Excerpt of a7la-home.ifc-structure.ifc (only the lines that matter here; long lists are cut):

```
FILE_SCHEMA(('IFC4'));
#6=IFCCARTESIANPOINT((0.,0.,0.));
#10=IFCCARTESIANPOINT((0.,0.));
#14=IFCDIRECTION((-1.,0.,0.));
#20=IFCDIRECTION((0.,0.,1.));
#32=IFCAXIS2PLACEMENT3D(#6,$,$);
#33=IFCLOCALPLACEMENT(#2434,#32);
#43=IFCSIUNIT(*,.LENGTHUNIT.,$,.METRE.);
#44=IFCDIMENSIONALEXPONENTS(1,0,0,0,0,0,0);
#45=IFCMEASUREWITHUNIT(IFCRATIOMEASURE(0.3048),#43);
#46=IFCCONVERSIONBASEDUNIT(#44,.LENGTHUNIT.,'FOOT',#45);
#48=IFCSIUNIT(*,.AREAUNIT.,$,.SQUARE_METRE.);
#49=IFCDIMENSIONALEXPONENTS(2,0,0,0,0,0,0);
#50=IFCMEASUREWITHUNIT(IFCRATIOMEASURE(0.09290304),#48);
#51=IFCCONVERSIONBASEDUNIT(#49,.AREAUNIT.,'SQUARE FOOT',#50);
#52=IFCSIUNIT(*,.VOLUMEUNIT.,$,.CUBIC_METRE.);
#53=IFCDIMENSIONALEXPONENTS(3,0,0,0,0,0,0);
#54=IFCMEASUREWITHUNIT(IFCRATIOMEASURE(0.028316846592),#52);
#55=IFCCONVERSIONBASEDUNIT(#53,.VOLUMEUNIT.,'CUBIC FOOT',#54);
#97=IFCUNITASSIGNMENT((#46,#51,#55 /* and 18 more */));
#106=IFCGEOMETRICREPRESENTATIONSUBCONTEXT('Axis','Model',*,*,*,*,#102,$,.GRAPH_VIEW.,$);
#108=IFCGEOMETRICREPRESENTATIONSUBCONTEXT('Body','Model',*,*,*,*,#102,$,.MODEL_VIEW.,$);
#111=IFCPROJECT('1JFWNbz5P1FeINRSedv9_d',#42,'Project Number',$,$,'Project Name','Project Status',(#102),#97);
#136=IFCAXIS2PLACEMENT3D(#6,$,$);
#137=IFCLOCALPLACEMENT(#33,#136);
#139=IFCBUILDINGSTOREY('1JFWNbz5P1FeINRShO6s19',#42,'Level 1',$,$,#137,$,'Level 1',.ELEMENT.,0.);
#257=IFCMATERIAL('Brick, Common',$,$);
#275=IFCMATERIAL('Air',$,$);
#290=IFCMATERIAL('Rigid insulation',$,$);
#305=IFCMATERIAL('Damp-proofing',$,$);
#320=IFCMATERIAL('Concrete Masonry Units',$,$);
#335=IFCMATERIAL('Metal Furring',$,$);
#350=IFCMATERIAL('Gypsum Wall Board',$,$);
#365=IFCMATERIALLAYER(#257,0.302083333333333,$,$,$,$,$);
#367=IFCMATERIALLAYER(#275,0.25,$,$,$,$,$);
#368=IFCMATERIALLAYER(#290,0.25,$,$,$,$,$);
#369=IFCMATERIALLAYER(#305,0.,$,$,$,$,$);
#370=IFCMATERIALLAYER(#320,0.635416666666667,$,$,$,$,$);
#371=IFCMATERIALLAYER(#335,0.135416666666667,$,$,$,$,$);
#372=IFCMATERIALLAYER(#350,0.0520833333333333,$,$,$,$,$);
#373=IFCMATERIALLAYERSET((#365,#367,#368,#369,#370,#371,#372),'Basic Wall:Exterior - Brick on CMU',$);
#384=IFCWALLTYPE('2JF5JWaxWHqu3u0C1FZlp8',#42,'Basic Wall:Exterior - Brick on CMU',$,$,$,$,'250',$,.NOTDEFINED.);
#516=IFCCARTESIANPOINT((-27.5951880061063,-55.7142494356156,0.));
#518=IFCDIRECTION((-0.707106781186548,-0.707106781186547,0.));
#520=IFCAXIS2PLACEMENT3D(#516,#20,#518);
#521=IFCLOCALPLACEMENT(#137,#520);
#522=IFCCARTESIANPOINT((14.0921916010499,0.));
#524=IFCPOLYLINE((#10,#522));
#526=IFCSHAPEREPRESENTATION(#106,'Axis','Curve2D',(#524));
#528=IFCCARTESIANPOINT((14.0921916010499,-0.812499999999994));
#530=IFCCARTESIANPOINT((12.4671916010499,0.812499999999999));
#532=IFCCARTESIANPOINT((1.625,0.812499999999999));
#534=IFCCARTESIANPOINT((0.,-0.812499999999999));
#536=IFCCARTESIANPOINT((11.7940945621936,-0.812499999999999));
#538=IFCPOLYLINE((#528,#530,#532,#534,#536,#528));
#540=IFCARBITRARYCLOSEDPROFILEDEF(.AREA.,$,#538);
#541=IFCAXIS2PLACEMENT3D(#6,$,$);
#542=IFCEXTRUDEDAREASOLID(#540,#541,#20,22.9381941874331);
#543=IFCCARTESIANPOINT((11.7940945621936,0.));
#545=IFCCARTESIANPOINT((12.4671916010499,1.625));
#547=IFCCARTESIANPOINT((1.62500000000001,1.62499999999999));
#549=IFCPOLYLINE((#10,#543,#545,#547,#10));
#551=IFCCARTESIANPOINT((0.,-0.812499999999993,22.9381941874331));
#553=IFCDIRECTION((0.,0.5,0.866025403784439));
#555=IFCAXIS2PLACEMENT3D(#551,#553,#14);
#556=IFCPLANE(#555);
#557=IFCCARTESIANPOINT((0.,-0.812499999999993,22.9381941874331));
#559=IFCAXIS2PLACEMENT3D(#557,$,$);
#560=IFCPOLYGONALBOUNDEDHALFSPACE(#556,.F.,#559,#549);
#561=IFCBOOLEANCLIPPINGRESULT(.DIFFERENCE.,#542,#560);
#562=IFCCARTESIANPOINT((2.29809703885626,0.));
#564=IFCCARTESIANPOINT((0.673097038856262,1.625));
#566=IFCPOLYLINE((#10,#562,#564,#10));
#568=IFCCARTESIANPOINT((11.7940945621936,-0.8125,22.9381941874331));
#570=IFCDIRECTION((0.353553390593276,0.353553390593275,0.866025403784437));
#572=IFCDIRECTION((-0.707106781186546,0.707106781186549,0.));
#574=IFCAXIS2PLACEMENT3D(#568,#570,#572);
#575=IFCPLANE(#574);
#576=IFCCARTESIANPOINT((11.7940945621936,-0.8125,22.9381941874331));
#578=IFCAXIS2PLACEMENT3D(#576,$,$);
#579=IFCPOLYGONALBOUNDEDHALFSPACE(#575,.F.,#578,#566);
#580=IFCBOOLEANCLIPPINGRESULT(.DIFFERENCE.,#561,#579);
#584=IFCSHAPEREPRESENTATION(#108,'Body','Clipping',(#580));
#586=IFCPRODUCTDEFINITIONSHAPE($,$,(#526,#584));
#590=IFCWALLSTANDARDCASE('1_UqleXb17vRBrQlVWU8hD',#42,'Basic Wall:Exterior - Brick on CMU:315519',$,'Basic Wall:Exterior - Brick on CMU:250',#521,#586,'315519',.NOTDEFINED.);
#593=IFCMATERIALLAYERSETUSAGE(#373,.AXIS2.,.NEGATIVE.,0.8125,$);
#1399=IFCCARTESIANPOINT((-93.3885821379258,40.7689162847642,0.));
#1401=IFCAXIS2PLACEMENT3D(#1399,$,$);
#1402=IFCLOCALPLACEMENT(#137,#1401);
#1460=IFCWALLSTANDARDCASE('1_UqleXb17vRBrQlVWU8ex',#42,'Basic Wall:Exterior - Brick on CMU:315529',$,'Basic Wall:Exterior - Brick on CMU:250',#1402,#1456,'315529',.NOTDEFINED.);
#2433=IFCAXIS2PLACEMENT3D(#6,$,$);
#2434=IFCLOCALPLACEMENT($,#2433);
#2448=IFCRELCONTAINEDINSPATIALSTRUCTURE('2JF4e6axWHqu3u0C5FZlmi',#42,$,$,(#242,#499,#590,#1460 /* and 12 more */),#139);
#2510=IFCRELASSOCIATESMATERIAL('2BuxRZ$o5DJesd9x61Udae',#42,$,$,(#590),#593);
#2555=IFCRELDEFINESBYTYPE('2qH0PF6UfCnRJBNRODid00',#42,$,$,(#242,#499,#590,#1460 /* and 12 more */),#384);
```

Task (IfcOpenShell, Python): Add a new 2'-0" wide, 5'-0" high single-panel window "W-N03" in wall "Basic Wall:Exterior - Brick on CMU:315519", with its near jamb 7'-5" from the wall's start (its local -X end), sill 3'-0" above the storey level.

```python
import numpy as np
import ifcopenshell
import ifcopenshell.api.feature
import ifcopenshell.api.geometry
import ifcopenshell.api.root
import ifcopenshell.api.spatial
import ifcopenshell.geom
import ifcopenshell.util.element
import ifcopenshell.util.placement
import ifcopenshell.util.representation
import ifcopenshell.util.shape
import ifcopenshell.util.unit

model = ifcopenshell.open("a7la-home.ifc-structure.ifc")
unit_scale = ifcopenshell.util.unit.calculate_unit_scale(model)
settings = ifcopenshell.geom.settings()


def volume(element):
    """Net volume in cubic metres, openings subtracted."""
    shape = ifcopenshell.geom.create_shape(settings, element)
    return ifcopenshell.util.shape.get_volume(shape.geometry)


wall = model.by_guid("1_UqleXb17vRBrQlVWU8hD")
storey = ifcopenshell.util.element.get_container(wall, ifc_class="IfcBuildingStorey")
context = ifcopenshell.util.representation.get_context(model, "Model", "Body", "MODEL_VIEW")
before = volume(wall)

width, height, from_end, sill = 0.6096, 1.524, 2.2606, 0.9144  # metres

# The wall runs along its own X axis, and the end named is its -X end.
wall_shape = ifcopenshell.geom.create_shape(settings, wall)
x, y, z = ifcopenshell.util.shape.get_vertices(wall_shape.geometry).T
start = x.min() + from_end
face, thickness = float(y.min()), float(y.max() - y.min())
wall_matrix = ifcopenshell.util.placement.get_local_placement(wall.ObjectPlacement)
level = ifcopenshell.util.placement.get_local_placement(storey.ObjectPlacement)[2, 3]


def in_wall(x, y):
    """Placement at x, y metres in the wall's axes, at sill height."""
    matrix = wall_matrix.copy()
    matrix[:, 3] = wall_matrix @ np.array([x / unit_scale, y / unit_scale, 0.0, 1.0])
    matrix[2, 3] = level + sill / unit_scale
    return matrix


# Opening: a box that overshoots both wall faces by 50 mm.
opening = ifcopenshell.api.root.create_entity(model, ifc_class="IfcOpeningElement", predefined_type="OPENING")
box = ifcopenshell.api.geometry.add_wall_representation(
    model, context=context, length=width, height=height, thickness=thickness + 0.1
)
ifcopenshell.api.geometry.assign_representation(model, product=opening, representation=box)
ifcopenshell.api.geometry.edit_object_placement(model, product=opening, matrix=in_wall(start, face - 0.05), is_si=False)
ifcopenshell.api.feature.add_feature(model, feature=opening, element=wall)

window = ifcopenshell.api.root.create_entity(model, ifc_class="IfcWindow", name="W-N03", predefined_type="WINDOW")
window.OverallWidth, window.OverallHeight = width / unit_scale, height / unit_scale
window.PartitioningType = "SINGLE_PANEL"
body = ifcopenshell.api.geometry.add_window_representation(
    model,
    context=context,
    overall_width=window.OverallWidth,
    overall_height=window.OverallHeight,
    partition_type="SINGLE_PANEL",
)
ifcopenshell.api.geometry.assign_representation(model, product=window, representation=body)
ifcopenshell.api.spatial.assign_container(model, products=[window], relating_structure=storey)
ifcopenshell.api.feature.add_filling(model, opening=opening, element=window)

# Centre the window in the wall's thickness.
ifcopenshell.api.geometry.edit_object_placement(model, product=window, matrix=in_wall(start, face), is_si=False)
window_shape = ifcopenshell.geom.create_shape(settings, window)
depth = ifcopenshell.util.shape.get_vertices(window_shape.geometry)[:, 1]
offset = face + thickness / 2 - (depth.min() + depth.max()) / 2
ifcopenshell.api.geometry.edit_object_placement(model, product=window, matrix=in_wall(start, offset), is_si=False)

after = volume(wall)

print(f"wall volume {before:.3f} -> {after:.3f} m3")

model.write("a7la-home.ifc-structure_v2.ifc")
```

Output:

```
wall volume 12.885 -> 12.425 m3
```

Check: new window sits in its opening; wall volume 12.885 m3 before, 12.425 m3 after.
